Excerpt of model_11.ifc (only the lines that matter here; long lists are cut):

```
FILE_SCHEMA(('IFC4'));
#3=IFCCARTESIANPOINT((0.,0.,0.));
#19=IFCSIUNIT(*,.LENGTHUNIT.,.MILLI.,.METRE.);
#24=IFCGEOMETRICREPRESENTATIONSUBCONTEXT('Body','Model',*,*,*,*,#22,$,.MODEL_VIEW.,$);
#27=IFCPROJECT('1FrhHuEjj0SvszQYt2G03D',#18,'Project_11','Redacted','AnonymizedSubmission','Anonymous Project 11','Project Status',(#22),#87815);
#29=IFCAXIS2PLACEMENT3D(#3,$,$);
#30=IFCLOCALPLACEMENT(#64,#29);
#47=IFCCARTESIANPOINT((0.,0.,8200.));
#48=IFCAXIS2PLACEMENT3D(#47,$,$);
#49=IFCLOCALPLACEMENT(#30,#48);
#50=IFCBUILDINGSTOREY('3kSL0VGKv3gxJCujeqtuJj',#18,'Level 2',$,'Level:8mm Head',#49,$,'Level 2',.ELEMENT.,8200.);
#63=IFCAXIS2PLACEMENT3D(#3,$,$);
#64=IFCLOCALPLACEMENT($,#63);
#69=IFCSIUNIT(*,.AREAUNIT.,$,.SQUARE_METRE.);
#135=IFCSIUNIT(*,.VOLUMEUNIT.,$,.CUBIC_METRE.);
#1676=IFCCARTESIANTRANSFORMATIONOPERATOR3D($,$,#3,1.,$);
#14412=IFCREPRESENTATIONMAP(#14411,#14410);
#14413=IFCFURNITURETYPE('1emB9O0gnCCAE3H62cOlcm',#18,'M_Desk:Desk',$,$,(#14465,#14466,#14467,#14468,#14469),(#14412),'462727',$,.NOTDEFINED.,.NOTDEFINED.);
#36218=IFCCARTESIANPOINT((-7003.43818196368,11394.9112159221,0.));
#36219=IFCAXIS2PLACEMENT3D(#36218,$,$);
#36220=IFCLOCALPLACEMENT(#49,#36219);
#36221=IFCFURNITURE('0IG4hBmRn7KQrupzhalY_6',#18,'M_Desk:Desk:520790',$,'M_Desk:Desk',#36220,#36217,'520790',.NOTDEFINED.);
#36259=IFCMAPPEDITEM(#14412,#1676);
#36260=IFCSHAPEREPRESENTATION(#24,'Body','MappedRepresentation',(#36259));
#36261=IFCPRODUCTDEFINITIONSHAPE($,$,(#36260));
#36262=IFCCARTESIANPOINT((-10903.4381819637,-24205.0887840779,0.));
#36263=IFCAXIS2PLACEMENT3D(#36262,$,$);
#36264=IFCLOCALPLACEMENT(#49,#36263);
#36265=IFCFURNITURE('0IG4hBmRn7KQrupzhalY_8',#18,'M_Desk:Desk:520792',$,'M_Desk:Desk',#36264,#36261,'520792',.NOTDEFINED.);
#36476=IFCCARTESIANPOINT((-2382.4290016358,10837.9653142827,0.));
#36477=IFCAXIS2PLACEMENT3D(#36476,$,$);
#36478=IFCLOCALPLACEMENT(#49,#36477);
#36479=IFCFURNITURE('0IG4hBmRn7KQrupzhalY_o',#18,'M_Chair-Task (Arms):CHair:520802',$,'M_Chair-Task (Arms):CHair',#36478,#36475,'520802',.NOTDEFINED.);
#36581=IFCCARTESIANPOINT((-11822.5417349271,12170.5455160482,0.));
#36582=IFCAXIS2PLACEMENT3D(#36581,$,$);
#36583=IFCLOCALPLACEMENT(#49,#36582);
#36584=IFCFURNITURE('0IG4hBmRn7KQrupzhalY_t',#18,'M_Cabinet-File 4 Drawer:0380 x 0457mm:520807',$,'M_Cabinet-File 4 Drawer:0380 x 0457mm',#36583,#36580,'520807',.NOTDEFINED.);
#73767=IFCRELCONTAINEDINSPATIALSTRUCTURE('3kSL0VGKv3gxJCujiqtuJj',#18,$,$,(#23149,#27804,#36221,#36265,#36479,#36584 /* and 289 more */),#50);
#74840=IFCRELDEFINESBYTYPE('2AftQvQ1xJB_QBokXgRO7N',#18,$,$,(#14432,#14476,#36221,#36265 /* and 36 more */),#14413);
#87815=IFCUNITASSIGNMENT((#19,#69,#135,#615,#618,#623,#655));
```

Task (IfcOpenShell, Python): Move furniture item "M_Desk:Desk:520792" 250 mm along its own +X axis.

```python
import ifcopenshell
import ifcopenshell.api.geometry
import ifcopenshell.util.placement

model = ifcopenshell.open("model_11.ifc")

item = model.by_guid("0IG4hBmRn7KQrupzhalY_8")
matrix = ifcopenshell.util.placement.get_local_placement(item.ObjectPlacement)
matrix[:3, 3] += matrix[:3, 0] * 250.0
ifcopenshell.api.geometry.edit_object_placement(model, product=item, matrix=matrix, is_si=False)

print(ifcopenshell.util.placement.get_local_placement(item.ObjectPlacement).round(3) + 0.0)

model.write("model_11_edited.ifc")
```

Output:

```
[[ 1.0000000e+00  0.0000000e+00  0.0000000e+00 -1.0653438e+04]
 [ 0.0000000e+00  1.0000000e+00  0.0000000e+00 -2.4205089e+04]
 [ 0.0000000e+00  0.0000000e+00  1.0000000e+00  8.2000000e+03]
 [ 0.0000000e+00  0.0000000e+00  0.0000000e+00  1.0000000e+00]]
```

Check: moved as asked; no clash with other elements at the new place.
